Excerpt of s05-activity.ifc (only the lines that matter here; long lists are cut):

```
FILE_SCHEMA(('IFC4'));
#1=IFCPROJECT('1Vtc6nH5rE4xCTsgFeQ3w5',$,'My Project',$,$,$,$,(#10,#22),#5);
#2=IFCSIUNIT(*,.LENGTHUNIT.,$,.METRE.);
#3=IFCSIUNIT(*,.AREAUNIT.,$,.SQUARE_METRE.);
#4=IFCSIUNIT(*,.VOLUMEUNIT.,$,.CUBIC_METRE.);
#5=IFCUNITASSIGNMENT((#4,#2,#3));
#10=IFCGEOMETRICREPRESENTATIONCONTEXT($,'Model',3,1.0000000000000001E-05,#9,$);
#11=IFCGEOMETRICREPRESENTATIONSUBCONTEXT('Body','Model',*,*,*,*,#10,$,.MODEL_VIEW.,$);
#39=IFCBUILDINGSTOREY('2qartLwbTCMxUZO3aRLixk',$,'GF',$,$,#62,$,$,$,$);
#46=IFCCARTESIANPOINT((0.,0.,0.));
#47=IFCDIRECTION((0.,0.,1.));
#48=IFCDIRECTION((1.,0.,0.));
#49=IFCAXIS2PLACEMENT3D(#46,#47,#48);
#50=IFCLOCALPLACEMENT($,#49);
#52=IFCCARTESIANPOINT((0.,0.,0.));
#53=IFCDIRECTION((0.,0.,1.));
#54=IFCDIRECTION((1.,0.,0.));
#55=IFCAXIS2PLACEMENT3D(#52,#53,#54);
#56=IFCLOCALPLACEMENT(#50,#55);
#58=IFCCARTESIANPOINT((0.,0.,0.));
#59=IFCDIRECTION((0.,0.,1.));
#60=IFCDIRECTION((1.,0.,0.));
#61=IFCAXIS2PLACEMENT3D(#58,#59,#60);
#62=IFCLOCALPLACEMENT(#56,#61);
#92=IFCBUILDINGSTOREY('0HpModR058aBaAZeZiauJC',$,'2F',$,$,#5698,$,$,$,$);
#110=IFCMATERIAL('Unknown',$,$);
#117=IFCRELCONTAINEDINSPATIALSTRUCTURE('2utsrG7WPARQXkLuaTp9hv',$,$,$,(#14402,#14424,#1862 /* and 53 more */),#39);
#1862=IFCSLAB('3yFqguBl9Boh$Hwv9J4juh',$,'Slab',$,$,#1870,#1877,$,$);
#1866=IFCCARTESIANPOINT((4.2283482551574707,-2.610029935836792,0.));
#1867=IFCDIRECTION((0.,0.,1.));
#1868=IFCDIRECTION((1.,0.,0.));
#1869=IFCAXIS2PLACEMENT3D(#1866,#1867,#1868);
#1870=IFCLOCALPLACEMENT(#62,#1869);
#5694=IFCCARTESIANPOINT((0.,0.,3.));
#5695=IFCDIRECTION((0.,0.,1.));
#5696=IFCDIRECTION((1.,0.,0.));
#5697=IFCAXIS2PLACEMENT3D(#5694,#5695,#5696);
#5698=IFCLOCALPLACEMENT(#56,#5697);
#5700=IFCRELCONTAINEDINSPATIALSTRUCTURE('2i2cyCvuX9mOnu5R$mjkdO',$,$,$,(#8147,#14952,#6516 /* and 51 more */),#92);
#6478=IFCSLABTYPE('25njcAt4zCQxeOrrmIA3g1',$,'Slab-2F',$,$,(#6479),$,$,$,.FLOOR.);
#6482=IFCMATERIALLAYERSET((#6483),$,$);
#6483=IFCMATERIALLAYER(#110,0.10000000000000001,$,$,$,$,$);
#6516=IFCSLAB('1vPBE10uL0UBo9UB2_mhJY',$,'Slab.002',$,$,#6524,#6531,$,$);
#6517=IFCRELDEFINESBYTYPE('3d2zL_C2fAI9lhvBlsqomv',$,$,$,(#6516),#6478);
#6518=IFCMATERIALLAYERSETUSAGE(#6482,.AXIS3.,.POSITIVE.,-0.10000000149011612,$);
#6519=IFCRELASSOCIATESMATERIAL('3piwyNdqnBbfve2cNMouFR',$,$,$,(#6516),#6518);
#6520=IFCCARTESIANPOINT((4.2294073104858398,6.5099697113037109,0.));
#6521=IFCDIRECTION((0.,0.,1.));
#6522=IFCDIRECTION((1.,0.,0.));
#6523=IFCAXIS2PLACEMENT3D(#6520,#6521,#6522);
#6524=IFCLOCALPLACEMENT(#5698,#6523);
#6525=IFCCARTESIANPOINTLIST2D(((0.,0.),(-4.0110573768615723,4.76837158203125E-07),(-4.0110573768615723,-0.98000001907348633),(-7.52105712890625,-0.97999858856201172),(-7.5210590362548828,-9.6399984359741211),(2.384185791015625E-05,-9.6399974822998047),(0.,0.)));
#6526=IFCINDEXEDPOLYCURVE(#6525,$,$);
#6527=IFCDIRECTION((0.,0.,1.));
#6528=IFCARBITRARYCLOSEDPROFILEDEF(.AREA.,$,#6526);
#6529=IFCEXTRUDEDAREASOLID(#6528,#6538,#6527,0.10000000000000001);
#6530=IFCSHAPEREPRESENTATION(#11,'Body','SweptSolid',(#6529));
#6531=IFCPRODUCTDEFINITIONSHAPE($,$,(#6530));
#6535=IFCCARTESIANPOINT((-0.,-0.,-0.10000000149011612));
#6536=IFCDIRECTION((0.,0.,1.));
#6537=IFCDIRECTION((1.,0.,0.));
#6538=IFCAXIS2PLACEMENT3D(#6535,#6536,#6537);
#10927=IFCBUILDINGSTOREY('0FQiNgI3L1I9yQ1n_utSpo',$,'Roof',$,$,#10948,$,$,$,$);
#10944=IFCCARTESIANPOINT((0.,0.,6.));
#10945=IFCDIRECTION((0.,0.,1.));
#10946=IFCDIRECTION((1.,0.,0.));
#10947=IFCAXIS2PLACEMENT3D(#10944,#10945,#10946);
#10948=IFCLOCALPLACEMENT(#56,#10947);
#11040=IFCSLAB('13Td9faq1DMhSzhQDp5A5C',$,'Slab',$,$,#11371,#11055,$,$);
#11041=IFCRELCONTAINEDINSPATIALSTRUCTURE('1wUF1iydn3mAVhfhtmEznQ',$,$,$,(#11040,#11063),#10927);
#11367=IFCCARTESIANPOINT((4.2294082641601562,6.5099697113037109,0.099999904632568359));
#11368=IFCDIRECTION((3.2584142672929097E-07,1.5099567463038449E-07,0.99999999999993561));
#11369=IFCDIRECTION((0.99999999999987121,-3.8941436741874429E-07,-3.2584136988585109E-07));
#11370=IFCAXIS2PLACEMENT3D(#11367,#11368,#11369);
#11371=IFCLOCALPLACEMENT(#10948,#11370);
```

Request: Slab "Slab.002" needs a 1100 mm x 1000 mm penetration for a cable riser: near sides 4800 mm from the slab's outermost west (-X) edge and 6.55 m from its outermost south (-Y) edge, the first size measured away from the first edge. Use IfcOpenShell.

```python
import numpy as np
import ifcopenshell
import ifcopenshell.api.feature
import ifcopenshell.api.geometry
import ifcopenshell.api.root
import ifcopenshell.geom
import ifcopenshell.util.placement
import ifcopenshell.util.representation
import ifcopenshell.util.shape
import ifcopenshell.util.unit

model = ifcopenshell.open("s05-activity.ifc")
unit_scale = ifcopenshell.util.unit.calculate_unit_scale(model)
settings = ifcopenshell.geom.settings()


def volume(element):
    """Net volume in cubic metres, openings subtracted."""
    shape = ifcopenshell.geom.create_shape(settings, element)
    return ifcopenshell.util.shape.get_volume(shape.geometry)


slab = model.by_id(6516)
before = volume(slab)

# Extent in the slab's own axes, in metres. The edges named are its -X and -Y sides.
slab_shape = ifcopenshell.geom.create_shape(settings, slab)
vertices = ifcopenshell.util.shape.get_vertices(slab_shape.geometry)
x_min, y_min, bottom = vertices.min(axis=0)
top = vertices[:, 2].max()

opening = ifcopenshell.api.root.create_entity(model, ifc_class="IfcOpeningElement", name="Cable riser opening", predefined_type="OPENING")
context = ifcopenshell.util.representation.get_context(model, "Model", "Body", "MODEL_VIEW")
width, depth = 1.1, 1
outline = [(0.0, 0.0), (width, 0.0), (width, depth), (0.0, depth), (0.0, 0.0)]
# Overshoot both faces by 50 mm so the cut is clean.
shape = ifcopenshell.api.geometry.add_slab_representation(
    model, context=context, depth=top - bottom + 0.1, polyline=outline
)
ifcopenshell.api.geometry.assign_representation(model, product=opening, representation=shape)

matrix = ifcopenshell.util.placement.get_local_placement(slab.ObjectPlacement)
matrix[:, 3] = matrix @ np.append(np.array([x_min + 4.8, y_min + 6.55, bottom - 0.05]) / unit_scale, 1.0)
ifcopenshell.api.geometry.edit_object_placement(model, product=opening, matrix=matrix, is_si=False)
ifcopenshell.api.feature.add_feature(model, feature=opening, element=slab)

after = volume(slab)

print(f"slab volume {before:.3f} -> {after:.3f} m3")

model.write("s05-activity_updated.ifc")
```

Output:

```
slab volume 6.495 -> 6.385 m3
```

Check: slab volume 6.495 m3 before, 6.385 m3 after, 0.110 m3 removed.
